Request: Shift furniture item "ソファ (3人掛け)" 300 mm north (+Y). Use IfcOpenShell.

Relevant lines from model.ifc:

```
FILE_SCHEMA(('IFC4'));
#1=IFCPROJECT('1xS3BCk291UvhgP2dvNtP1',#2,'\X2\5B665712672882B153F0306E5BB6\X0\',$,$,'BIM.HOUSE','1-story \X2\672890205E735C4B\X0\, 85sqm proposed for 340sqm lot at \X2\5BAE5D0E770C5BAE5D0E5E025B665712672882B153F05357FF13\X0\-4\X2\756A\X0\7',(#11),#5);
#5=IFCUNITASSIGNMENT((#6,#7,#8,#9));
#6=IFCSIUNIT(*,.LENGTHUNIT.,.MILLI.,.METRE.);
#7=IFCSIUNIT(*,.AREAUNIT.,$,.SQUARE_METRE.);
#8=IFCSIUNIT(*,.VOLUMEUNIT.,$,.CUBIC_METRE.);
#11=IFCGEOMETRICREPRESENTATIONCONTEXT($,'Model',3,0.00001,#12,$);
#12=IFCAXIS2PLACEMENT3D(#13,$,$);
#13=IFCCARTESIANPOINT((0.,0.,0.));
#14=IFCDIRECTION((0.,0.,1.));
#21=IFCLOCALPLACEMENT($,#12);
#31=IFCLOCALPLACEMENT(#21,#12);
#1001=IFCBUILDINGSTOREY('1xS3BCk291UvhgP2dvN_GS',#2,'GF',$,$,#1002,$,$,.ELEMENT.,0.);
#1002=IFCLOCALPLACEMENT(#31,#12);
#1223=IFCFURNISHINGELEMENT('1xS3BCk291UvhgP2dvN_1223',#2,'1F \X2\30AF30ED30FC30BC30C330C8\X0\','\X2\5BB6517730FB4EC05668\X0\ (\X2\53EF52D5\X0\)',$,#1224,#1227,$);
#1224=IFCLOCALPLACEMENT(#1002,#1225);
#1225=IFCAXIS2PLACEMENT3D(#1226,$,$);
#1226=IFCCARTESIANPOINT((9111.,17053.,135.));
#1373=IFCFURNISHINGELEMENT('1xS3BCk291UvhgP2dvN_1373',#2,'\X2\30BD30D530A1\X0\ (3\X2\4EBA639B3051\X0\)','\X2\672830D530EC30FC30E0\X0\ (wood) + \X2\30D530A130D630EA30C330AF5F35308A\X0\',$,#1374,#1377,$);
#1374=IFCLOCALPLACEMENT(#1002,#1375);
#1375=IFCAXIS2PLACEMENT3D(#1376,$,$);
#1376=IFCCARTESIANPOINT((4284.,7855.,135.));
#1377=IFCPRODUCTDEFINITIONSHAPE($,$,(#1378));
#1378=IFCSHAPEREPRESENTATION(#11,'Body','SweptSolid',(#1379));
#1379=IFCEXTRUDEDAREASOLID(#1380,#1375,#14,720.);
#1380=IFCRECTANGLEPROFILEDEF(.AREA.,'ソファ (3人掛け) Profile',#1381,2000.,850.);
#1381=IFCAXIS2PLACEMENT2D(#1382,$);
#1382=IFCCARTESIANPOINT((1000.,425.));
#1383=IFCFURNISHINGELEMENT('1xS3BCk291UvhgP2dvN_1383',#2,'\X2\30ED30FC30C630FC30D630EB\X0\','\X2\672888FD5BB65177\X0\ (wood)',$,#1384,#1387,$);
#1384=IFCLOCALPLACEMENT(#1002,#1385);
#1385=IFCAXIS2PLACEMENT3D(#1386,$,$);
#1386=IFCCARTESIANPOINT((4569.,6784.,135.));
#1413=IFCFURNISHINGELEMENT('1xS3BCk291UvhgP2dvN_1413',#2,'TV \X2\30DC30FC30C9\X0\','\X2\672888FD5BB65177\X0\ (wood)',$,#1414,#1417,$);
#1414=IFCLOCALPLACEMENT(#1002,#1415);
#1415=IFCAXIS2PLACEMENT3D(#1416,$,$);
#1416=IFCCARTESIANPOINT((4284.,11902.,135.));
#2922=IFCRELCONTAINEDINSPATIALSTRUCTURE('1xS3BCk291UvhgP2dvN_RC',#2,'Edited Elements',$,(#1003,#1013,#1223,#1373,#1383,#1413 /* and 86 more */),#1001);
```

```python
import ifcopenshell
import ifcopenshell.api.geometry
import ifcopenshell.util.placement
import ifcopenshell.util.unit

model = ifcopenshell.open("model.ifc")
unit_scale = ifcopenshell.util.unit.calculate_unit_scale(model)

item = model.by_guid("1xS3BCk291UvhgP2dvN_1373")
matrix = ifcopenshell.util.placement.get_local_placement(item.ObjectPlacement)
matrix[1, 3] += 0.3 / unit_scale
ifcopenshell.api.geometry.edit_object_placement(model, product=item, matrix=matrix, is_si=False)

print(ifcopenshell.util.placement.get_local_placement(item.ObjectPlacement).round(3) + 0.0)

model.write("model_updated.ifc")
```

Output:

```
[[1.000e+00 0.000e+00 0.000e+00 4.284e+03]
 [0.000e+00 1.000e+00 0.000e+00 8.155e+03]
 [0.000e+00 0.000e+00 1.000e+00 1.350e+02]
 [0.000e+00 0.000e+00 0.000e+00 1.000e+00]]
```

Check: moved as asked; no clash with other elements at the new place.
